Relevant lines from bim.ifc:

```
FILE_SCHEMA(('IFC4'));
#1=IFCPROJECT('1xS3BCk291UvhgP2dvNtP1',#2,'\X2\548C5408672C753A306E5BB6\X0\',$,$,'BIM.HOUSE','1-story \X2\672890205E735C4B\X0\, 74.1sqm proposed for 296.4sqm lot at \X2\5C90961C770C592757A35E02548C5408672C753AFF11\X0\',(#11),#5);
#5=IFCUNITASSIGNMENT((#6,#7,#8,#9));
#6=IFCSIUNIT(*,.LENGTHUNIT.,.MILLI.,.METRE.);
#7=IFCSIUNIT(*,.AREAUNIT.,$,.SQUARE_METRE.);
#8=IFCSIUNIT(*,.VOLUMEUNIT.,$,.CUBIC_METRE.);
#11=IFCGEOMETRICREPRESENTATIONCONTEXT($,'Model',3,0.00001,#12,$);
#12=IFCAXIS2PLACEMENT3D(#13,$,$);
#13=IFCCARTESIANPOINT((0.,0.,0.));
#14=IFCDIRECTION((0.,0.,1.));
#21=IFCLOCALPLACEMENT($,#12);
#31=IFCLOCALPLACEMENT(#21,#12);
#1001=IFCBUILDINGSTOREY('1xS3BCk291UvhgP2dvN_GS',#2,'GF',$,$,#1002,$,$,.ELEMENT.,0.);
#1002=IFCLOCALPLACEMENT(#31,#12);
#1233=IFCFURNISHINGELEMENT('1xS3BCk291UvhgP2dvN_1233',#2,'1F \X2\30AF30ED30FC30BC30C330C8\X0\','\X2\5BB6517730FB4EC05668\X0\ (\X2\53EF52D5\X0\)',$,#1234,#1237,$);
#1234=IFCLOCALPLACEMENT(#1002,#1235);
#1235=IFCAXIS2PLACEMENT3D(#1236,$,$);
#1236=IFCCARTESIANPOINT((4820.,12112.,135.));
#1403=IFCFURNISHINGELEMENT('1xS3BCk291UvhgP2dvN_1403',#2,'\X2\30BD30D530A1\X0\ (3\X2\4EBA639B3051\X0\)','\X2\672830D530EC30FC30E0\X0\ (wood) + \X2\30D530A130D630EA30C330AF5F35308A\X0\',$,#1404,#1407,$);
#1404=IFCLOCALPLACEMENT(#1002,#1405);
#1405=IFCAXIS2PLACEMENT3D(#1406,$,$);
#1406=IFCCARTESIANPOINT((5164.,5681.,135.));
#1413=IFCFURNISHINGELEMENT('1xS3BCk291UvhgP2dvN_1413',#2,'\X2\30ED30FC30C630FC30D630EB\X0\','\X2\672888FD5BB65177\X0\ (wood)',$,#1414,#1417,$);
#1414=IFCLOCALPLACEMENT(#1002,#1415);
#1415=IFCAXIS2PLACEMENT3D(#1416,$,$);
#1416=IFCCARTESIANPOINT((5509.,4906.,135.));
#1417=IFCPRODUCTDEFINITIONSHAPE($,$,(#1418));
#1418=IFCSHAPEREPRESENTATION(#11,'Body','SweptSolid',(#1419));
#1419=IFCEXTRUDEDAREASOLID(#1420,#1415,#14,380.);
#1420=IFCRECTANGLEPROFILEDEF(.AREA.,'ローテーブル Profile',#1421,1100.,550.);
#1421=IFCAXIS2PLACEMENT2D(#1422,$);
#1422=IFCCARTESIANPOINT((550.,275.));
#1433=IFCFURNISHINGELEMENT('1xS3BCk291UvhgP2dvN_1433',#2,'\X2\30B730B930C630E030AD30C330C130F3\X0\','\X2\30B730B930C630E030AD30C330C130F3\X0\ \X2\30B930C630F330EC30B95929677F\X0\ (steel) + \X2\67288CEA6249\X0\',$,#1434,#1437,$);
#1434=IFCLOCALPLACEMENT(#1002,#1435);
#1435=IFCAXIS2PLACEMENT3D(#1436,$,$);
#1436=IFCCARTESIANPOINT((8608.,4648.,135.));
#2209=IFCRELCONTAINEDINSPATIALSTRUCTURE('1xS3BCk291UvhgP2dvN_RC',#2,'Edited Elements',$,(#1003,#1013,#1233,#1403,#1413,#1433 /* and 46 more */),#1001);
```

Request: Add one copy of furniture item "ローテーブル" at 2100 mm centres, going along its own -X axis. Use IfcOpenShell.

```python
import ifcopenshell
import ifcopenshell.api.geometry
import ifcopenshell.api.root
import ifcopenshell.util.element
import ifcopenshell.util.placement

model = ifcopenshell.open("bim.ifc")


def reuse_history(source, copy):
    """copy_class also copies each property set's owner history, people and application; keep the originals."""
    for rel in copy.IsDefinedBy:
        if rel.is_a("IfcRelDefinesByProperties") and (history := rel.RelatingPropertyDefinition.OwnerHistory):
            rel.RelatingPropertyDefinition.OwnerHistory = source.OwnerHistory
            ifcopenshell.util.element.remove_deep2(model, history)


source = model.by_guid("1xS3BCk291UvhgP2dvN_1413")
base = ifcopenshell.util.placement.get_local_placement(source.ObjectPlacement)
step = -base[:3, 0] * 2100.0

for i in range(1, 2):
    copy = ifcopenshell.api.root.copy_class(model, product=source)
    copy.Representation = ifcopenshell.util.element.copy_deep(
        model, source.Representation, exclude=["IfcGeometricRepresentationContext", "IfcRepresentationMap"]
    )
    reuse_history(source, copy)
    matrix = base.copy()
    matrix[:3, 3] += i * step
    print("added at", matrix[:3, 3].round(3) + 0.0)
    ifcopenshell.api.geometry.edit_object_placement(model, product=copy, matrix=matrix, is_si=False)

model.write("bim_v2.ifc")
```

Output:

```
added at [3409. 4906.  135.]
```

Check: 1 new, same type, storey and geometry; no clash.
